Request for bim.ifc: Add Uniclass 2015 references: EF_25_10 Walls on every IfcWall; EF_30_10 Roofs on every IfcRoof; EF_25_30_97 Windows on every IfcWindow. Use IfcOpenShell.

First a look at what the model holds.

```python
import ifcopenshell

model = ifcopenshell.open("bim.ifc")
print(model.schema)
print("classifications:", [c.Name for c in model.by_type("IfcClassification")])
for ifc_class in ("IfcDoor", "IfcRoof", "IfcStair", "IfcWall", "IfcWindow"):
    print(ifc_class, len(model.by_type(ifc_class)))
```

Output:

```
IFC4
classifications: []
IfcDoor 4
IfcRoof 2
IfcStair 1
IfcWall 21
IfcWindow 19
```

```python
import ifcopenshell
import ifcopenshell.api.classification

model = ifcopenshell.open("bim.ifc")

system = ifcopenshell.api.classification.add_classification(model, classification="Uniclass 2015")

codes = {
    "IfcWall": ("EF_25_10", "Walls"),
    "IfcRoof": ("EF_30_10", "Roofs"),
    "IfcWindow": ("EF_25_30_97", "Windows"),
}
for ifc_class, (code, name) in codes.items():
    products = model.by_type(ifc_class)
    ifcopenshell.api.classification.add_reference(
        model, products=products, classification=system, identification=code, name=name
    )
    print(code, len(products))

model.write("bim_rev.ifc")
```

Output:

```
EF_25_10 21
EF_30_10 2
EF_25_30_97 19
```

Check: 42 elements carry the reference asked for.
